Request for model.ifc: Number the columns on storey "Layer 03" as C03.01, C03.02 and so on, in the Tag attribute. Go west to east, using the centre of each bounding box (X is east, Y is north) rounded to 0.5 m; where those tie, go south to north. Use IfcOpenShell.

First a look at what the model holds.

```python
import ifcopenshell
import ifcopenshell.util.element
import ifcopenshell.util.placement

model = ifcopenshell.open("model.ifc")
print(model.schema)
storey = next(s for s in model.by_type("IfcBuildingStorey") if s.Name == "Layer 03")
columns = [e for e in ifcopenshell.util.element.get_decomposition(storey) if e.is_a("IfcColumn")]
for e in sorted(columns, key=lambda e: e.id()):
    origin = ifcopenshell.util.placement.get_local_placement(e.ObjectPlacement)[:3, 3]
    print(e.id(), e.Tag, e.Name, origin.round(2) + 0.0, sep=" | ")
```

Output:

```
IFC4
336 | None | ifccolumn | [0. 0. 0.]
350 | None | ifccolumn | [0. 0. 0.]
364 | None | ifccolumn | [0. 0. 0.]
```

```python
import ifcopenshell
import ifcopenshell.geom
import ifcopenshell.util.element
import ifcopenshell.util.shape

model = ifcopenshell.open("model.ifc")
settings = ifcopenshell.geom.settings()
settings.set("use-world-coords", True)


def centre(element):
    shape = ifcopenshell.geom.create_shape(settings, element)
    return ifcopenshell.util.shape.get_bbox_centroid(shape.geometry)


storey = next(s for s in model.by_type("IfcBuildingStorey") if s.Name == "Layer 03")
columns = [e for e in ifcopenshell.util.element.get_decomposition(storey) if e.is_a("IfcColumn")]

# Insertion points can sit at a corner or the storey origin, so sort by the geometry (in metres).
centres = {e: centre(e) for e in columns}
columns.sort(key=lambda e: (round(centres[e][0] / 0.5), centres[e][1]))

for i, e in enumerate(columns, start=1):
    number = f"C03.{i:02d}"
    e.Tag = number
    print(e.id(), number)

model.write("model-out.ifc")
```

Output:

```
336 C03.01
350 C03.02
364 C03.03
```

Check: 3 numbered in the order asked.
